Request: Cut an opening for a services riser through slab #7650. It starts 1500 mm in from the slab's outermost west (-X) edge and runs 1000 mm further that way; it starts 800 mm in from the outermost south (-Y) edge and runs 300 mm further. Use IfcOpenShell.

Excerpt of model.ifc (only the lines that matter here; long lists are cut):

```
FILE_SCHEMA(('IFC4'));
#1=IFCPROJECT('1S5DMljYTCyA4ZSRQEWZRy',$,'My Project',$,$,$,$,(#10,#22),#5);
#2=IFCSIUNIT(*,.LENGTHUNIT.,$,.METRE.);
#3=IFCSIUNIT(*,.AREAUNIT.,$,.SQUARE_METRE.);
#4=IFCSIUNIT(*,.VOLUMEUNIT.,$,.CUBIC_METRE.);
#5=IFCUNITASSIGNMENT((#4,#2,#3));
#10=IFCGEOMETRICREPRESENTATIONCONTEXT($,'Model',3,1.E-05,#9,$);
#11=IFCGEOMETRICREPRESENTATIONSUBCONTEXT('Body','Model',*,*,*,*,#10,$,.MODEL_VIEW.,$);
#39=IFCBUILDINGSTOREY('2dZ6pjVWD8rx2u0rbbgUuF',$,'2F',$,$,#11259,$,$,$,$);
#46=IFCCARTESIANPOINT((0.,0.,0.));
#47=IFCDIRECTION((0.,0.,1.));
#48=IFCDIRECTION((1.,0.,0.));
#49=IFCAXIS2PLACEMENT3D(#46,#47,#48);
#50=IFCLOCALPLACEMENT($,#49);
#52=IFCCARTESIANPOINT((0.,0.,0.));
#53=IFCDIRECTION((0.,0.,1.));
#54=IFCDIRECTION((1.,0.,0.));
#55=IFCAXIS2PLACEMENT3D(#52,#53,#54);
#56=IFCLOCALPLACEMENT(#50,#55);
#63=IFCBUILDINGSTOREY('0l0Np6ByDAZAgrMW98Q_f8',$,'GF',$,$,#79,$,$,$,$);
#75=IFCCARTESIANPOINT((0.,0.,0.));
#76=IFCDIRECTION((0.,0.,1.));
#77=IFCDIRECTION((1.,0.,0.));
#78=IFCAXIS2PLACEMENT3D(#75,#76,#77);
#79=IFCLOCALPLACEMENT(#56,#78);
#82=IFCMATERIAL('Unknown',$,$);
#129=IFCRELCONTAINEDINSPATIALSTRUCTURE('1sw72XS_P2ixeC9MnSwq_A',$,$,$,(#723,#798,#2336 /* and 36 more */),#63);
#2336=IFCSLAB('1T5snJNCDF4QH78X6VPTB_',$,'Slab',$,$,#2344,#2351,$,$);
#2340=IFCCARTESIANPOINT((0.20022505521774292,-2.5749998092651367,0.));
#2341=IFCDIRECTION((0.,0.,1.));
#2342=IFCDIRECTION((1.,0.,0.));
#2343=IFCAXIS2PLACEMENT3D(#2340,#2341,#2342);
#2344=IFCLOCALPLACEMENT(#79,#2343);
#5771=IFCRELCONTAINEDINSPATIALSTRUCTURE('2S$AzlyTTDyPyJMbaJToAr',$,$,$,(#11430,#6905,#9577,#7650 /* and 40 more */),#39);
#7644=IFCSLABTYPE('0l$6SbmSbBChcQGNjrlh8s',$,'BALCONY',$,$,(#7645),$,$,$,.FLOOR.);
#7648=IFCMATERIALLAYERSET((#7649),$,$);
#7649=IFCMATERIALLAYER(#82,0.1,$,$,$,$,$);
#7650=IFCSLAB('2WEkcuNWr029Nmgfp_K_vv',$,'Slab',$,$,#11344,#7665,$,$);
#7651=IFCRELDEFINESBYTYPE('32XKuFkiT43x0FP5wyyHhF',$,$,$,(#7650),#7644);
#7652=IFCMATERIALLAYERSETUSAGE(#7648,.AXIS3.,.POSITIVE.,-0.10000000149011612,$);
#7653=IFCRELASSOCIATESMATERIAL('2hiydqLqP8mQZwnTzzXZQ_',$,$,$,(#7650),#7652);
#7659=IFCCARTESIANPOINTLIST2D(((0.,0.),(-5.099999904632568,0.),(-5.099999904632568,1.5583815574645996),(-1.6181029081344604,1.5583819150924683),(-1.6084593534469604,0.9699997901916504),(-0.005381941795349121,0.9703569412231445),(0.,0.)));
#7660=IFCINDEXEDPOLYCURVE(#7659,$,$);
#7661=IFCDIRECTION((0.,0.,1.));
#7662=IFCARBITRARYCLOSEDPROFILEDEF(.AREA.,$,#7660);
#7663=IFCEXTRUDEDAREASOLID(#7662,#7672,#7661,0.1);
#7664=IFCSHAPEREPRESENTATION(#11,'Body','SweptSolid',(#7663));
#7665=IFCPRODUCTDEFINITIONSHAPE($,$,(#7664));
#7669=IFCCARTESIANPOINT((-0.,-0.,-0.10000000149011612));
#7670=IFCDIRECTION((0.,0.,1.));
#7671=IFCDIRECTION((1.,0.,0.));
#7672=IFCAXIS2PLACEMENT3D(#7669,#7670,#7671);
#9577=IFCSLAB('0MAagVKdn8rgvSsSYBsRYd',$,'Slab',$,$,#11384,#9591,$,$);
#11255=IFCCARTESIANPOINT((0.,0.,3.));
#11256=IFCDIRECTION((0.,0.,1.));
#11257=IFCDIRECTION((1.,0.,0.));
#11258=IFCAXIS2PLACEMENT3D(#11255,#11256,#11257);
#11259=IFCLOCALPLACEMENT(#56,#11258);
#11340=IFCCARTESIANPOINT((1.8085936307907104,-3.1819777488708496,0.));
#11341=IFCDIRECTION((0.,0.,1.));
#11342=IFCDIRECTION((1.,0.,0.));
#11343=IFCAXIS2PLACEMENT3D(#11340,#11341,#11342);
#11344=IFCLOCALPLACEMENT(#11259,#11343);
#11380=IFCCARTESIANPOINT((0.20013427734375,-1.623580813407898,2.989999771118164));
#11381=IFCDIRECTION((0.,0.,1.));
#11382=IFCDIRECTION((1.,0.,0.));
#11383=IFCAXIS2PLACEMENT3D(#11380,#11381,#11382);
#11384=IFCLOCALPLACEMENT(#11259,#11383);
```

```python
import numpy as np
import ifcopenshell
import ifcopenshell.api.feature
import ifcopenshell.api.geometry
import ifcopenshell.api.root
import ifcopenshell.geom
import ifcopenshell.util.placement
import ifcopenshell.util.representation
import ifcopenshell.util.shape
import ifcopenshell.util.unit

model = ifcopenshell.open("model.ifc")
unit_scale = ifcopenshell.util.unit.calculate_unit_scale(model)
settings = ifcopenshell.geom.settings()


def volume(element):
    """Net volume in cubic metres, openings subtracted."""
    shape = ifcopenshell.geom.create_shape(settings, element)
    return ifcopenshell.util.shape.get_volume(shape.geometry)


slab = model.by_guid("2WEkcuNWr029Nmgfp_K_vv")
before = volume(slab)

# Extent in the slab's own axes, in metres. The edges named are its -X and -Y sides.
slab_shape = ifcopenshell.geom.create_shape(settings, slab)
vertices = ifcopenshell.util.shape.get_vertices(slab_shape.geometry)
x_min, y_min, bottom = vertices.min(axis=0)
top = vertices[:, 2].max()

opening = ifcopenshell.api.root.create_entity(model, ifc_class="IfcOpeningElement", name="Services riser opening", predefined_type="OPENING")
context = ifcopenshell.util.representation.get_context(model, "Model", "Body", "MODEL_VIEW")
width, depth = 1, 0.3
outline = [(0.0, 0.0), (width, 0.0), (width, depth), (0.0, depth), (0.0, 0.0)]
# Overshoot both faces by 50 mm so the cut is clean.
shape = ifcopenshell.api.geometry.add_slab_representation(
    model, context=context, depth=top - bottom + 0.1, polyline=outline
)
ifcopenshell.api.geometry.assign_representation(model, product=opening, representation=shape)

matrix = ifcopenshell.util.placement.get_local_placement(slab.ObjectPlacement)
matrix[:, 3] = matrix @ np.append(np.array([x_min + 1.5, y_min + 0.8, bottom - 0.05]) / unit_scale, 1.0)
ifcopenshell.api.geometry.edit_object_placement(model, product=opening, matrix=matrix, is_si=False)
ifcopenshell.api.feature.add_feature(model, feature=opening, element=slab)

after = volume(slab)

print(f"slab volume {before:.3f} -> {after:.3f} m3")

model.write("model_v2.ifc")
```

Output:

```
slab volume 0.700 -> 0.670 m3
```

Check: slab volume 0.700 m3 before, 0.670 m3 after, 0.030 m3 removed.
